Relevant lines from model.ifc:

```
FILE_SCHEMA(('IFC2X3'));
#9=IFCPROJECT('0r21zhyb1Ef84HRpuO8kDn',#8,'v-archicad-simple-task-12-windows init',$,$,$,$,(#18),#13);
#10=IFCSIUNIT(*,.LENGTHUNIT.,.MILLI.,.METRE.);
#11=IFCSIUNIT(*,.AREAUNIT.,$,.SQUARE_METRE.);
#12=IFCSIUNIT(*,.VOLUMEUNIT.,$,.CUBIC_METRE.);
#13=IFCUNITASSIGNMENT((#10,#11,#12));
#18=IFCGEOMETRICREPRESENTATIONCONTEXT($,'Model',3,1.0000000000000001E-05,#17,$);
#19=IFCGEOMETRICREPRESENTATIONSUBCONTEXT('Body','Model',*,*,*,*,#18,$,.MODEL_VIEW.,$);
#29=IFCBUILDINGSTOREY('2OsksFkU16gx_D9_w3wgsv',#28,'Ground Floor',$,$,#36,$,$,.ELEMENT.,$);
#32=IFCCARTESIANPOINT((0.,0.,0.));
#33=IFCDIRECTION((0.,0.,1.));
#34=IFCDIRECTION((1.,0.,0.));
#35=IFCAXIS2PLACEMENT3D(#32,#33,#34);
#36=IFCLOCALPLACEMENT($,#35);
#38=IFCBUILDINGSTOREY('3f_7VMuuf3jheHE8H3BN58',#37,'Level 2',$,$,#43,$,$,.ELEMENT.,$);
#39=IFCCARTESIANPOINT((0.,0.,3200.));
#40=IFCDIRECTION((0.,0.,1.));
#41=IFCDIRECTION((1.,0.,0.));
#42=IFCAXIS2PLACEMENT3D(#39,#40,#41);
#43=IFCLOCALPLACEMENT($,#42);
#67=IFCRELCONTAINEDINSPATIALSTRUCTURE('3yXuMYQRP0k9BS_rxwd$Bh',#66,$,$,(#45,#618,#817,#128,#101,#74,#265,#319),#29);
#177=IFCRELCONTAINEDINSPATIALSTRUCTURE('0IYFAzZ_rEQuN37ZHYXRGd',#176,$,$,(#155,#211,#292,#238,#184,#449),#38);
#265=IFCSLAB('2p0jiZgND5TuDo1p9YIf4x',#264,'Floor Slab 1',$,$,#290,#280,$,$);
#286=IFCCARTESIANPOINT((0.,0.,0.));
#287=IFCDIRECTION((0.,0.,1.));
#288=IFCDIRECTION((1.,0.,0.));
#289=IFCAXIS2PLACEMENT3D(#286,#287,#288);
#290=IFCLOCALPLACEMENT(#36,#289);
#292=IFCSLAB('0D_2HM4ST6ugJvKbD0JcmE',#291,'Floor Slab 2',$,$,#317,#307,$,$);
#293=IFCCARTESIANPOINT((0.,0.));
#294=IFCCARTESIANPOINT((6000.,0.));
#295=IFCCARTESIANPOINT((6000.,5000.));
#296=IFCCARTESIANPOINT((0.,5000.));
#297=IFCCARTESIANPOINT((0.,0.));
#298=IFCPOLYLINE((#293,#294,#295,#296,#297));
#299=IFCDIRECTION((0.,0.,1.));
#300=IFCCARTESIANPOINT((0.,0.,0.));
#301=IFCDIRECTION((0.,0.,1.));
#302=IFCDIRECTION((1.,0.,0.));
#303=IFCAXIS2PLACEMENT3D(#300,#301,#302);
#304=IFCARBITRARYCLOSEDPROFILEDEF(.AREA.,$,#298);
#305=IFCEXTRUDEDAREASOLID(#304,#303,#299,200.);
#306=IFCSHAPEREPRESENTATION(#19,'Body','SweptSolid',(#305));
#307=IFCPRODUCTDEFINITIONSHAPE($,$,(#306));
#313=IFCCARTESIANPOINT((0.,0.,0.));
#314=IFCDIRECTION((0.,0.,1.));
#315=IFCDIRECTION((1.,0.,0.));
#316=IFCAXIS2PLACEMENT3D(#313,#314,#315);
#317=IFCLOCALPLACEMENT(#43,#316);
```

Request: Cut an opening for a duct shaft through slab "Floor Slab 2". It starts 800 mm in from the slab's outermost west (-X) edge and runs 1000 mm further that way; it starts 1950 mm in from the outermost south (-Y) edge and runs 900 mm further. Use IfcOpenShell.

```python
import numpy as np
import ifcopenshell
import ifcopenshell.api.feature
import ifcopenshell.api.geometry
import ifcopenshell.api.root
import ifcopenshell.geom
import ifcopenshell.util.placement
import ifcopenshell.util.representation
import ifcopenshell.util.shape
import ifcopenshell.util.unit

model = ifcopenshell.open("model.ifc")
unit_scale = ifcopenshell.util.unit.calculate_unit_scale(model)
settings = ifcopenshell.geom.settings()


def volume(element):
    """Net volume in cubic metres, openings subtracted."""
    shape = ifcopenshell.geom.create_shape(settings, element)
    return ifcopenshell.util.shape.get_volume(shape.geometry)


slab = model.by_guid("0D_2HM4ST6ugJvKbD0JcmE")
before = volume(slab)

# Extent in the slab's own axes, in metres. The edges named are its -X and -Y sides.
slab_shape = ifcopenshell.geom.create_shape(settings, slab)
vertices = ifcopenshell.util.shape.get_vertices(slab_shape.geometry)
x_min, y_min, bottom = vertices.min(axis=0)
top = vertices[:, 2].max()

opening = ifcopenshell.api.root.create_entity(model, ifc_class="IfcOpeningElement", name="Duct shaft opening")
context = ifcopenshell.util.representation.get_context(model, "Model", "Body", "MODEL_VIEW")
width, depth = 1, 0.9
outline = [(0.0, 0.0), (width, 0.0), (width, depth), (0.0, depth), (0.0, 0.0)]
# Overshoot both faces by 50 mm so the cut is clean.
shape = ifcopenshell.api.geometry.add_slab_representation(
    model, context=context, depth=top - bottom + 0.1, polyline=outline
)
ifcopenshell.api.geometry.assign_representation(model, product=opening, representation=shape)

matrix = ifcopenshell.util.placement.get_local_placement(slab.ObjectPlacement)
matrix[:, 3] = matrix @ np.append(np.array([x_min + 0.8, y_min + 1.95, bottom - 0.05]) / unit_scale, 1.0)
ifcopenshell.api.geometry.edit_object_placement(model, product=opening, matrix=matrix, is_si=False)
ifcopenshell.api.feature.add_feature(model, feature=opening, element=slab)

after = volume(slab)

print(f"slab volume {before:.3f} -> {after:.3f} m3")

model.write("model_updated.ifc")
```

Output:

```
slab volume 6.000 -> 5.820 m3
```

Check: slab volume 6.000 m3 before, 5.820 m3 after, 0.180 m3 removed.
